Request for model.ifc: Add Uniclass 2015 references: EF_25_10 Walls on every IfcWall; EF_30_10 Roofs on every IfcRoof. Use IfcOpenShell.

First a look at what the model holds.

```python
import ifcopenshell

model = ifcopenshell.open("model.ifc")
print(model.schema)
print("classifications:", [c.Name for c in model.by_type("IfcClassification")])
for ifc_class in ("IfcDoor", "IfcRoof", "IfcStair", "IfcWall", "IfcWindow"):
    print(ifc_class, len(model.by_type(ifc_class)))
```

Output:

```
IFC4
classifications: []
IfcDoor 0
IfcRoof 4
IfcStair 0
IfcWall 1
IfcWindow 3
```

```python
import ifcopenshell
import ifcopenshell.api.classification

model = ifcopenshell.open("model.ifc")

system = ifcopenshell.api.classification.add_classification(model, classification="Uniclass 2015")

codes = {
    "IfcWall": ("EF_25_10", "Walls"),
    "IfcRoof": ("EF_30_10", "Roofs"),
}
for ifc_class, (code, name) in codes.items():
    products = model.by_type(ifc_class)
    ifcopenshell.api.classification.add_reference(
        model, products=products, classification=system, identification=code, name=name
    )
    print(code, len(products))

model.write("model_edited.ifc")
```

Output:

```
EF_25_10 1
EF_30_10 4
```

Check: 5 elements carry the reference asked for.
